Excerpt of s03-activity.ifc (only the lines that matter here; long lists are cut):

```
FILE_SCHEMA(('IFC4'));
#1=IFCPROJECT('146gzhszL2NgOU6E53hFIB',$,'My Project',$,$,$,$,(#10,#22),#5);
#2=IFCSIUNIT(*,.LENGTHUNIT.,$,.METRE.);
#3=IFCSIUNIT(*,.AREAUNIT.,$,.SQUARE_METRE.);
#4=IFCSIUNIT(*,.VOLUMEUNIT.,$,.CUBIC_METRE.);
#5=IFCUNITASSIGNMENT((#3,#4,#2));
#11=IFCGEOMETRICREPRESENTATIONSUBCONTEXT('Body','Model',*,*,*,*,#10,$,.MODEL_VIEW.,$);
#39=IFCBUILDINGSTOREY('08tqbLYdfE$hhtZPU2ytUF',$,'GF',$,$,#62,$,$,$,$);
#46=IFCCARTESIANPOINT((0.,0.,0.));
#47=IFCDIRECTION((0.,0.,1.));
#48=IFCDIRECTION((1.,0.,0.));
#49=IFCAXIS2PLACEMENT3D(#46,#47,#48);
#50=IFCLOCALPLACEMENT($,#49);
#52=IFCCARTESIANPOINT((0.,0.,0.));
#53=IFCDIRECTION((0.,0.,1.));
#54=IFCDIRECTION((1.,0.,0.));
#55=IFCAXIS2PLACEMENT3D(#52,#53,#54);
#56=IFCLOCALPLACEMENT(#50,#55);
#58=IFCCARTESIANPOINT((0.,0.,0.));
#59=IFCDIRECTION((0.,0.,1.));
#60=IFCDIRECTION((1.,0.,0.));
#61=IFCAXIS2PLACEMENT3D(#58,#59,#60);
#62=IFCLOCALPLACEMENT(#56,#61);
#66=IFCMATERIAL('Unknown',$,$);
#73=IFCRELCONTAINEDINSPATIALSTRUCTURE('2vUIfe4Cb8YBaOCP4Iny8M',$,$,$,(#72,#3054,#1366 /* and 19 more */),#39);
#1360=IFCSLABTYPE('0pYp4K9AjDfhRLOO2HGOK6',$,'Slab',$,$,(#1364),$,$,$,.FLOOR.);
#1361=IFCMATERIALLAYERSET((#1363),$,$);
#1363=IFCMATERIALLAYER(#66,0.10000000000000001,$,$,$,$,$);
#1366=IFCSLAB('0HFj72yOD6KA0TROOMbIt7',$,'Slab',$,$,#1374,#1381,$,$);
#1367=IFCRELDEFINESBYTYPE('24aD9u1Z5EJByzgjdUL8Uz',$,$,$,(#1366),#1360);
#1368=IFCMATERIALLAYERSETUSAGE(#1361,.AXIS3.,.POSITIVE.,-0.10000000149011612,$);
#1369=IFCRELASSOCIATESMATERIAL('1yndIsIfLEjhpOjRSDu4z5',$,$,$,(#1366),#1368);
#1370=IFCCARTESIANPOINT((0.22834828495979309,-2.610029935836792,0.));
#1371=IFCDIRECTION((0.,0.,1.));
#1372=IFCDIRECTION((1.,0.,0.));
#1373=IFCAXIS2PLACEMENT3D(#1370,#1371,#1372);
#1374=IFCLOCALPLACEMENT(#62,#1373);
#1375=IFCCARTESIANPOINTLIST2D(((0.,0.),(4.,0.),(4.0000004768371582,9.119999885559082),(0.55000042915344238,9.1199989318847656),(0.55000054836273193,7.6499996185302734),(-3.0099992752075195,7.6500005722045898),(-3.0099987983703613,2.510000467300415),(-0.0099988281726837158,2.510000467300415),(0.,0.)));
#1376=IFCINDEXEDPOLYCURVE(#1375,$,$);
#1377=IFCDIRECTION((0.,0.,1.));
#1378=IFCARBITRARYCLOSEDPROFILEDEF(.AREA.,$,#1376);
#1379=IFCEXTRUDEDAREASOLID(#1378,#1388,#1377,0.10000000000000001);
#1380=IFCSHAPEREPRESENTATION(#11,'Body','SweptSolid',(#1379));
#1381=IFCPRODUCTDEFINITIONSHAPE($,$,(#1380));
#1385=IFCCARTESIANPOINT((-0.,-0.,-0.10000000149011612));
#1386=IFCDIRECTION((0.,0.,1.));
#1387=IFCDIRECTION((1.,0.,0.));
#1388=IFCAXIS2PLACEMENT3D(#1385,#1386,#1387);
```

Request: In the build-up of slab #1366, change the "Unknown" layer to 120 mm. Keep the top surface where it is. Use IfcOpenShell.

```python
import ifcopenshell
import ifcopenshell.util.element
import ifcopenshell.util.representation

model = ifcopenshell.open("s03-activity.ifc")

layer_set = model.by_id(1361)
layer = next(l for l in layer_set.MaterialLayers if l.Material and l.Material.Name == "Unknown")
change = 0.12 - layer.LayerThickness
layer.LayerThickness += change

# Geometry does not follow the layer set by itself.
slabs = [e for e in ifcopenshell.util.element.get_elements_by_material(model, layer_set) if e.is_a("IfcSlab")]
for slab in sorted(slabs, key=lambda e: e.id()):
    body = ifcopenshell.util.representation.get_representation(slab, "Model", "Body")
    solid = body.Items[0]
    old_depth = solid.Depth
    solid.Depth += change
    # Extruded upwards: lower the start of the extrusion so the top stays.
    x, y, z = solid.Position.Location.Coordinates
    solid.Position.Location = model.createIfcCartesianPoint((x, y, z - change))
    print(slab.id(), f"{old_depth:g} -> {solid.Depth:g}")

# The layers are counted up from the underside, which has moved.
for usage in {ifcopenshell.util.element.get_material(slab) for slab in slabs}:
    usage.OffsetFromReferenceLine -= change

model.write("s03-activity-out.ifc")
```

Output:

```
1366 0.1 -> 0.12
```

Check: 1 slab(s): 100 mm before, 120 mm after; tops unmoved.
